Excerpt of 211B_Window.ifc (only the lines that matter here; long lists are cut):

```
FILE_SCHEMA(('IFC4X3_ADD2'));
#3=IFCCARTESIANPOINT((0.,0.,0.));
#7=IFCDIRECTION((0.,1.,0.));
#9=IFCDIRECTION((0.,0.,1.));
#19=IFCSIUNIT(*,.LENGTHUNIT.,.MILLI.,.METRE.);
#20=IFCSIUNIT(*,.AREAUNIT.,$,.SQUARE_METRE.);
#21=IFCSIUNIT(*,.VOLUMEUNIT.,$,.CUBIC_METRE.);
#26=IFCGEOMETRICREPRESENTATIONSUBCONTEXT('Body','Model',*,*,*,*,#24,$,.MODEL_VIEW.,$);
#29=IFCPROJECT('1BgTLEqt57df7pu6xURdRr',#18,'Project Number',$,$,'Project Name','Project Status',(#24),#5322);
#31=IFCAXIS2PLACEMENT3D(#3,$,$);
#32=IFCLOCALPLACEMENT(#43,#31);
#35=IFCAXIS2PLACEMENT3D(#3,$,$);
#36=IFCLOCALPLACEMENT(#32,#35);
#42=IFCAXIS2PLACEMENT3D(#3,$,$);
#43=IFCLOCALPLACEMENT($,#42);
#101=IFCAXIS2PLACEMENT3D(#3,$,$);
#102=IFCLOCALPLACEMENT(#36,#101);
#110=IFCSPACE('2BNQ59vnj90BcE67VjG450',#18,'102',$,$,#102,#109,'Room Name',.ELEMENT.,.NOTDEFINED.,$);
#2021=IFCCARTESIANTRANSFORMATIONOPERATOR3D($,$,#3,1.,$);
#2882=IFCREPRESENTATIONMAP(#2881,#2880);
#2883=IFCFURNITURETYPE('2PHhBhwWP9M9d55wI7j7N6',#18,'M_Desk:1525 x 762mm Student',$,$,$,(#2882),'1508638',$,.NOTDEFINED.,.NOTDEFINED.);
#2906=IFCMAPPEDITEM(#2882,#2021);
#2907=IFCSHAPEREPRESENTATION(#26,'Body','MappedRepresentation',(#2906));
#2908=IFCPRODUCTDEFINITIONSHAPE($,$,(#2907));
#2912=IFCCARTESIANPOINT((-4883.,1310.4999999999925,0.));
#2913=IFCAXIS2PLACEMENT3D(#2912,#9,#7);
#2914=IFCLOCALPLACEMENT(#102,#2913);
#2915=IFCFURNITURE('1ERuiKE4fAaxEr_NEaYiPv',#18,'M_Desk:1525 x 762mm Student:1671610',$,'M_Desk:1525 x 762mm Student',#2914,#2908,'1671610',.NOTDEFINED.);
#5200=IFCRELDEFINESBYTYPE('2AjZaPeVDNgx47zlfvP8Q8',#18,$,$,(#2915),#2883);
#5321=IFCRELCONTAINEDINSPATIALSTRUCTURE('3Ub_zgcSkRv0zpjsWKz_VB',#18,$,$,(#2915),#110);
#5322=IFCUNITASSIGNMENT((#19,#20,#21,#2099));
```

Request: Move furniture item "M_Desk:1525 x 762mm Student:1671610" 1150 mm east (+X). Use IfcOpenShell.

```python
import ifcopenshell
import ifcopenshell.api.geometry
import ifcopenshell.util.placement

model = ifcopenshell.open("211B_Window.ifc")

item = model.by_guid("1ERuiKE4fAaxEr_NEaYiPv")
matrix = ifcopenshell.util.placement.get_local_placement(item.ObjectPlacement)
matrix[0, 3] += 1150.0
ifcopenshell.api.geometry.edit_object_placement(model, product=item, matrix=matrix, is_si=False)

print(ifcopenshell.util.placement.get_local_placement(item.ObjectPlacement).round(3) + 0.0)

model.write("211B_Window_edited.ifc")
```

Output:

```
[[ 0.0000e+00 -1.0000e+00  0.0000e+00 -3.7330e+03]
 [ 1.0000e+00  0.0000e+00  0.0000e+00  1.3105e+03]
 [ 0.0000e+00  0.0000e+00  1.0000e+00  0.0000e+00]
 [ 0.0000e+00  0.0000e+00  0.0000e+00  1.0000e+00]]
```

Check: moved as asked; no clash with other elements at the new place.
